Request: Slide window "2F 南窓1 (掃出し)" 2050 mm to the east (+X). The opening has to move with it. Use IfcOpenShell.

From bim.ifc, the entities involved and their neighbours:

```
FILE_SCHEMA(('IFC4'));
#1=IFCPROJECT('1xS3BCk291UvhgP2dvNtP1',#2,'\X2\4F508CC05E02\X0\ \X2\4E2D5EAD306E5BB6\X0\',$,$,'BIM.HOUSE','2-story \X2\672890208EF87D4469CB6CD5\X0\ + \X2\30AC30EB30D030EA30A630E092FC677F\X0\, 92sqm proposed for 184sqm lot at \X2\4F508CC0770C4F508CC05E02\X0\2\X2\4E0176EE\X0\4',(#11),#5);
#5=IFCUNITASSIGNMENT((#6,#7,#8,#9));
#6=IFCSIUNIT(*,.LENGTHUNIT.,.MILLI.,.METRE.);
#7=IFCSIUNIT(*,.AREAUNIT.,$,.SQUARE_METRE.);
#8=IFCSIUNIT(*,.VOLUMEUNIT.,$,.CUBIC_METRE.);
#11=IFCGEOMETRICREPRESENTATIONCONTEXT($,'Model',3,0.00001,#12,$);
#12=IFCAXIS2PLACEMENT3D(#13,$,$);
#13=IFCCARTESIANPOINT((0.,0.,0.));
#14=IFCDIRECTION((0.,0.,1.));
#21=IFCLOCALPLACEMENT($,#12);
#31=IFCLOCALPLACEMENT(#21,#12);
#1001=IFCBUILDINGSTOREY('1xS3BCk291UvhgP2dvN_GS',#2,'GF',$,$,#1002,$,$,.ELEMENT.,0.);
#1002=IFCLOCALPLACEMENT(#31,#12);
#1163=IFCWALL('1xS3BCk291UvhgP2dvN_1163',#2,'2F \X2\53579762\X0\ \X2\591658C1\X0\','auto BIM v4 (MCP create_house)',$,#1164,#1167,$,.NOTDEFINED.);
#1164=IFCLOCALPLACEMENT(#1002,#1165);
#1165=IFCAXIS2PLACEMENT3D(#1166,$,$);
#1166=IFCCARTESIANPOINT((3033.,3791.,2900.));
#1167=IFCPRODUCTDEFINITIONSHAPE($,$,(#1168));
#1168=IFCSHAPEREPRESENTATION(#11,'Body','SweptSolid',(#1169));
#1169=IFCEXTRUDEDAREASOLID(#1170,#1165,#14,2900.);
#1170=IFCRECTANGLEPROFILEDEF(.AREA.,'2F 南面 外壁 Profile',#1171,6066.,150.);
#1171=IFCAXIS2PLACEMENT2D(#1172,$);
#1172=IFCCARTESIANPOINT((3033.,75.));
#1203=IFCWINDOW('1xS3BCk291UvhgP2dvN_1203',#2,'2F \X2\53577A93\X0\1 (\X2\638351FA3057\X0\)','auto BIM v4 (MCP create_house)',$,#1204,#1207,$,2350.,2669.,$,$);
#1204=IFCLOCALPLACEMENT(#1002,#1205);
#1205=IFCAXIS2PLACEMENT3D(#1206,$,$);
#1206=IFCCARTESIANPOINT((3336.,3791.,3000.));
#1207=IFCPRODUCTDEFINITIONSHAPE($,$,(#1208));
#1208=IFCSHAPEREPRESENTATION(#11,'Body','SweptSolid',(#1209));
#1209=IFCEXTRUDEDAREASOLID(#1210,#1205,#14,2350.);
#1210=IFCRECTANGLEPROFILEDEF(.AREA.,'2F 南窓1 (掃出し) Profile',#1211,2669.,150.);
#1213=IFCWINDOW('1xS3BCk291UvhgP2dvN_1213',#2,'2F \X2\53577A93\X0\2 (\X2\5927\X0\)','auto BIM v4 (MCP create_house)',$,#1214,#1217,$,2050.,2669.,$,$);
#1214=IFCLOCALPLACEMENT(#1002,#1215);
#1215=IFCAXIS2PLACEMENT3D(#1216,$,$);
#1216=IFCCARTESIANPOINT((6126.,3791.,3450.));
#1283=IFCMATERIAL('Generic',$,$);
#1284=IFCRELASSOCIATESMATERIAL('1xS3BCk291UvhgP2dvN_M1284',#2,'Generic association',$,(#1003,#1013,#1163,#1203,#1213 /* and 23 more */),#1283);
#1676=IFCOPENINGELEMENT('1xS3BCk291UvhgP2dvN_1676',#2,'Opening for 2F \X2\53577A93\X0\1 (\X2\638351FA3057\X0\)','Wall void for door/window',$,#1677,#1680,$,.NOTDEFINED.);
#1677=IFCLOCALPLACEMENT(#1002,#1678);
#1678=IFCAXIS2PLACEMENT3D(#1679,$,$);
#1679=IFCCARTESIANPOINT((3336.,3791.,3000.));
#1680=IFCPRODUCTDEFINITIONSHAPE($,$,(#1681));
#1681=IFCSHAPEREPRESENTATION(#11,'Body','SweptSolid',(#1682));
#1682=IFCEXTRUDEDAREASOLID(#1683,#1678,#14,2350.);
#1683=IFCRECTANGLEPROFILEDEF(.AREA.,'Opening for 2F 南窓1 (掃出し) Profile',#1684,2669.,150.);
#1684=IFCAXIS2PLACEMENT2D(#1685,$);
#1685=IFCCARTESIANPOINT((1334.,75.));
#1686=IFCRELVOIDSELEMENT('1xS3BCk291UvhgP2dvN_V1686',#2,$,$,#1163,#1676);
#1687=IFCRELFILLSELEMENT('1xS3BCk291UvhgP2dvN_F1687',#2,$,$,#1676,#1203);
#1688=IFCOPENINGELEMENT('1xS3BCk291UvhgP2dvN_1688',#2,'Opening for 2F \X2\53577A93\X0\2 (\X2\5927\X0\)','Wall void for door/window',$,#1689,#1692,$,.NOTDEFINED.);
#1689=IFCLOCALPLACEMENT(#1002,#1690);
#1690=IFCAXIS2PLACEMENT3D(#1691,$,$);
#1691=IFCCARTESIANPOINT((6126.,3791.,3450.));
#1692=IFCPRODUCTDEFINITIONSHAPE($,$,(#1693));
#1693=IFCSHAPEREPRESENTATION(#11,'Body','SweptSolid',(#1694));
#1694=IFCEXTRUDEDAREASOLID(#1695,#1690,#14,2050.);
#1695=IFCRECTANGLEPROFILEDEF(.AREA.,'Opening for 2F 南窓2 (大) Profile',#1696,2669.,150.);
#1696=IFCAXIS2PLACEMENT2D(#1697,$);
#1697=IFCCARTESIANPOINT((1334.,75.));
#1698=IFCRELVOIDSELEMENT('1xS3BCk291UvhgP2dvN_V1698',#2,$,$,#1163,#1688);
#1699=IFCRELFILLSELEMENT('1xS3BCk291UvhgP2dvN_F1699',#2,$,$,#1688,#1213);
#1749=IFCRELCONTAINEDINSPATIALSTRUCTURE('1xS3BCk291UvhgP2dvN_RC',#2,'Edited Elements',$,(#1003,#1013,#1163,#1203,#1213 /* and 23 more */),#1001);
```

```python
import ifcopenshell
import ifcopenshell.api.geometry
import ifcopenshell.util.placement

model = ifcopenshell.open("bim.ifc")

window = model.by_guid("1xS3BCk291UvhgP2dvN_1203")
opening = window.FillsVoids[0].RelatingOpeningElement
wall = opening.VoidsElements[0].RelatingBuildingElement

wall_matrix = ifcopenshell.util.placement.get_local_placement(wall.ObjectPlacement)
shift = wall_matrix[:3, 0] * 2050.0
before = ifcopenshell.util.placement.get_local_placement(window.ObjectPlacement)[:3, 3].copy()

# The window is not placed relative to its opening, so move both.
for product in (opening, window):
    matrix = ifcopenshell.util.placement.get_local_placement(product.ObjectPlacement)
    matrix[:3, 3] += shift
    ifcopenshell.api.geometry.edit_object_placement(model, product=product, matrix=matrix, is_si=False)

after = ifcopenshell.util.placement.get_local_placement(window.ObjectPlacement)[:3, 3]
print("window moved by", (after - before).round(3) + 0.0)

model.write("bim_rev.ifc")
```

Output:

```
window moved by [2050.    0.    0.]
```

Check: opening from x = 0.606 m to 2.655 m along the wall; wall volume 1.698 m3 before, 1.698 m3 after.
